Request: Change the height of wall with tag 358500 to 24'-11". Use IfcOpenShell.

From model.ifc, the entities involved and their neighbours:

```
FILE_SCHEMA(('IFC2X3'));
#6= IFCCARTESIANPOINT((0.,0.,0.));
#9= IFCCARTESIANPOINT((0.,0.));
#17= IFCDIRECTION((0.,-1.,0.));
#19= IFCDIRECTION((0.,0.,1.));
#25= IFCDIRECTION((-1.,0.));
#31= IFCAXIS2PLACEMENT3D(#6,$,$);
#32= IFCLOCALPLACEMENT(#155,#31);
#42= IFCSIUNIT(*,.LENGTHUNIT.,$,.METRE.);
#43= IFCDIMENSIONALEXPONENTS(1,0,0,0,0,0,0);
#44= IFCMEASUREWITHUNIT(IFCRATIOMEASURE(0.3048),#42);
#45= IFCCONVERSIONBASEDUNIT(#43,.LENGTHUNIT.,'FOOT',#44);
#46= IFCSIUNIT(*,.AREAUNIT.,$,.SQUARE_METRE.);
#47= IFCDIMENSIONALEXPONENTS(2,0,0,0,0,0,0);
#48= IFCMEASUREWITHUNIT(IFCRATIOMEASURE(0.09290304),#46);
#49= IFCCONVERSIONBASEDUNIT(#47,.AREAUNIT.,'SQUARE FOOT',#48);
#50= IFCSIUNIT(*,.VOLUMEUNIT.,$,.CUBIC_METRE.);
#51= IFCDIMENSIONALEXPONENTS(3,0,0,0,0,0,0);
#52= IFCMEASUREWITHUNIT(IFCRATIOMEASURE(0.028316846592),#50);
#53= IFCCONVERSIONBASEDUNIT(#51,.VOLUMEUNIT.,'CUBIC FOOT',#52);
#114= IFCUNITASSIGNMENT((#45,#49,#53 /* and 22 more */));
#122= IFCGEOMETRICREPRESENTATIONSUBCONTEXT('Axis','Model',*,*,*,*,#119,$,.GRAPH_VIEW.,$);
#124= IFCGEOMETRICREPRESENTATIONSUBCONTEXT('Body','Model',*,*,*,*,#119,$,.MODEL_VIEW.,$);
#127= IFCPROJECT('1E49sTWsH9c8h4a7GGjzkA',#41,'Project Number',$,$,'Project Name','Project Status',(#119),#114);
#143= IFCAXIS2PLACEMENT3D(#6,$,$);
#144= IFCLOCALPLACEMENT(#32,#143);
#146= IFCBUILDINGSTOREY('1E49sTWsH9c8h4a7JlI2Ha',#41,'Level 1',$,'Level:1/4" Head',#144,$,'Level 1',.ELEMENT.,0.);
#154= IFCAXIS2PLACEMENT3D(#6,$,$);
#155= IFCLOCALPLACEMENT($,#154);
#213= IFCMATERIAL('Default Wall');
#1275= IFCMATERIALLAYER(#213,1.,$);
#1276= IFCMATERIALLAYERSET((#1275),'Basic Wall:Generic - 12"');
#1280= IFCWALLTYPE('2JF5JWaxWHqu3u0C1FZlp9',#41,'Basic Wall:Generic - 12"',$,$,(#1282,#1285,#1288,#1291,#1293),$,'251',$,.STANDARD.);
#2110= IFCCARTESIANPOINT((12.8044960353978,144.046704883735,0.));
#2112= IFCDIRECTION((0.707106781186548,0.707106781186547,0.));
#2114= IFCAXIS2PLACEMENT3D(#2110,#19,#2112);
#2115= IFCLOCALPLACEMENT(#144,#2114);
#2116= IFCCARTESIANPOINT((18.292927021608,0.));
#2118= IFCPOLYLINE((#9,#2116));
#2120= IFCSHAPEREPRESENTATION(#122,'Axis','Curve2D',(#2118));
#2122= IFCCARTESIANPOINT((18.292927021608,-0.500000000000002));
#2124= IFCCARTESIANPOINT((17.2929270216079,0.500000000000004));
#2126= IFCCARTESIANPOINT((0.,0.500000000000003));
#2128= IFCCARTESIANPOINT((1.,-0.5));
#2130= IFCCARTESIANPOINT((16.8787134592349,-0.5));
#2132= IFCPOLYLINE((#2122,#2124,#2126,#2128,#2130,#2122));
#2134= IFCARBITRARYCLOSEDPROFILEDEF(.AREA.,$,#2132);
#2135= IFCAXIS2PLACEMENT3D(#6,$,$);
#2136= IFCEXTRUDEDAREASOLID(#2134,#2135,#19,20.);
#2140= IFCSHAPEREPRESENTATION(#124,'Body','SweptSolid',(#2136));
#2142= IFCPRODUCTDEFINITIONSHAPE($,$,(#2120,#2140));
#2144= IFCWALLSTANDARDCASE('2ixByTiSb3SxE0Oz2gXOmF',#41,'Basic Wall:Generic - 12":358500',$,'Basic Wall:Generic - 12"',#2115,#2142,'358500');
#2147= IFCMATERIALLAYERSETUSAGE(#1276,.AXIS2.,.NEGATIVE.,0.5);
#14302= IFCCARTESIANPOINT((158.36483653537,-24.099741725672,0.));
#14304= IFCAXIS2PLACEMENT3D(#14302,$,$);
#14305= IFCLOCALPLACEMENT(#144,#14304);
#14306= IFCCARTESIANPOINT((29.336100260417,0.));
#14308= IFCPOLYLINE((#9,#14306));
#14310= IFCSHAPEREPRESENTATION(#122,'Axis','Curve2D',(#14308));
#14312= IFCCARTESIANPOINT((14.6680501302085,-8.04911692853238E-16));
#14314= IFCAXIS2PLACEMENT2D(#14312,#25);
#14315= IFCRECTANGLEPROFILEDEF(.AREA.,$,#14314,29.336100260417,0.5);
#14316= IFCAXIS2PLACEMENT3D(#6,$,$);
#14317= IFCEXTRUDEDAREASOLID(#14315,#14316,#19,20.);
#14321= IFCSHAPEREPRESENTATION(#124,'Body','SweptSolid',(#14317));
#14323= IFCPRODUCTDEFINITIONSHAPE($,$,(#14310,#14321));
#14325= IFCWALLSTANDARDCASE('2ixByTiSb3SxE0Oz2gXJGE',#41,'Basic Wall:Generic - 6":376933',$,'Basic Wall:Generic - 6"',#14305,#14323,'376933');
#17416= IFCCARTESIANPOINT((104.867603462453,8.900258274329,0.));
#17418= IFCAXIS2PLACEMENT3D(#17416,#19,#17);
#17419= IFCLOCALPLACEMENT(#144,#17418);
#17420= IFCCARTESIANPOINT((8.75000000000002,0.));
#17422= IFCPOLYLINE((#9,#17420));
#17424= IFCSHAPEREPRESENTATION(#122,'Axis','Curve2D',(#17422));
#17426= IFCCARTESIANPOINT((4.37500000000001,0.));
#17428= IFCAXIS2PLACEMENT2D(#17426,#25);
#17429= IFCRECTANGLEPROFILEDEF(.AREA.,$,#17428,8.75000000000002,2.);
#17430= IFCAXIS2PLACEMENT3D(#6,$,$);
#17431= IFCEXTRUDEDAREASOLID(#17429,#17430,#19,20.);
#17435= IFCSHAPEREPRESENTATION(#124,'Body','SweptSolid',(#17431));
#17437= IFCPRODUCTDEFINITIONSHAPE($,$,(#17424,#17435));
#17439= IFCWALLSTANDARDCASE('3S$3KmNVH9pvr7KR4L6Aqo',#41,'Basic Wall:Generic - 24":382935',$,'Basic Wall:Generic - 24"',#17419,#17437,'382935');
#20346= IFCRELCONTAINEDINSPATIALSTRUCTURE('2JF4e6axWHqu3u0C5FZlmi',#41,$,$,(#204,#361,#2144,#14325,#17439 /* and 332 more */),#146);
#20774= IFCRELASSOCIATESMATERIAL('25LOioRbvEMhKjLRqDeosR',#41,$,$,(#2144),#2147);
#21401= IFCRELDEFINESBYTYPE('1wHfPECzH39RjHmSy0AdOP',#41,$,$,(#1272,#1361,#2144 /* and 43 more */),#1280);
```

```python
import ifcopenshell
import ifcopenshell.geom
import ifcopenshell.util.representation
import ifcopenshell.util.shape
import ifcopenshell.util.unit

model = ifcopenshell.open("model.ifc")
unit_scale = ifcopenshell.util.unit.calculate_unit_scale(model)
settings = ifcopenshell.geom.settings()


def volume(element):
    """Net volume in cubic metres, openings subtracted."""
    shape = ifcopenshell.geom.create_shape(settings, element)
    return ifcopenshell.util.shape.get_volume(shape.geometry)


wall = model.by_id(2144)
before = volume(wall)

body = ifcopenshell.util.representation.get_representation(wall, "Model", "Body")
solid = body.Items[0]
old_height = solid.Depth
solid.Depth = 299 * 0.0254 / unit_scale
after = volume(wall)

print(f"height {old_height:g} -> {solid.Depth:g}, volume {before:.3f} -> {after:.3f} m3")

model.write("model_edited.ifc")
```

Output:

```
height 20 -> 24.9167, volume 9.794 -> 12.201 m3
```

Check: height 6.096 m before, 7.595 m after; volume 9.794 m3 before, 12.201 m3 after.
